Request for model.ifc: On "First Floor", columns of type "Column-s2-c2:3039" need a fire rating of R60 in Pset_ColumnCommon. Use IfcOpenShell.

First a look at what the model holds.

```python
import ifcopenshell
import ifcopenshell.util.element

model = ifcopenshell.open("model.ifc")
print(model.schema)
storey = next(s for s in model.by_type("IfcBuildingStorey") if s.Name == "First Floor")
columns = [e for e in ifcopenshell.util.element.get_decomposition(storey) if e.is_a("IfcColumn")]
seen = {}
for e in columns:
    element_type = ifcopenshell.util.element.get_type(e)
    key = (element_type.Name if element_type != e and element_type else None, ifcopenshell.util.element.get_pset(e, "Pset_ColumnCommon", "FireRating"))
    seen[key] = seen.get(key, 0) + 1
for (name, value), count in sorted(seen.items(), key=str):
    print(count, "x", name, "|", value)
```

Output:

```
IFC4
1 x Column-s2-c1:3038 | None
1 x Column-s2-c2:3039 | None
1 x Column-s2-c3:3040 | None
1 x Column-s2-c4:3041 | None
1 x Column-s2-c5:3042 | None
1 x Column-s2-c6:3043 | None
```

```python
import ifcopenshell
import ifcopenshell.api.pset
import ifcopenshell.util.element

model = ifcopenshell.open("model.ifc")

storey = next(s for s in model.by_type("IfcBuildingStorey") if s.Name == "First Floor")
columns = [e for e in ifcopenshell.util.element.get_decomposition(storey) if e.is_a("IfcColumn")]

count = 0
for e in columns:
    element_type = ifcopenshell.util.element.get_type(e)
    if element_type in (None, e) or element_type.Name != "Column-s2-c2:3039":
        continue
    # add_pset returns the element's existing set when there is one.
    pset = ifcopenshell.api.pset.add_pset(model, product=e, name="Pset_ColumnCommon")
    ifcopenshell.api.pset.edit_pset(model, pset=pset, properties={"FireRating": "R60"})
    count += 1

print(count, "columns updated")

model.write("model_updated.ifc")
```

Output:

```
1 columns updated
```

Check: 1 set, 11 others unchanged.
